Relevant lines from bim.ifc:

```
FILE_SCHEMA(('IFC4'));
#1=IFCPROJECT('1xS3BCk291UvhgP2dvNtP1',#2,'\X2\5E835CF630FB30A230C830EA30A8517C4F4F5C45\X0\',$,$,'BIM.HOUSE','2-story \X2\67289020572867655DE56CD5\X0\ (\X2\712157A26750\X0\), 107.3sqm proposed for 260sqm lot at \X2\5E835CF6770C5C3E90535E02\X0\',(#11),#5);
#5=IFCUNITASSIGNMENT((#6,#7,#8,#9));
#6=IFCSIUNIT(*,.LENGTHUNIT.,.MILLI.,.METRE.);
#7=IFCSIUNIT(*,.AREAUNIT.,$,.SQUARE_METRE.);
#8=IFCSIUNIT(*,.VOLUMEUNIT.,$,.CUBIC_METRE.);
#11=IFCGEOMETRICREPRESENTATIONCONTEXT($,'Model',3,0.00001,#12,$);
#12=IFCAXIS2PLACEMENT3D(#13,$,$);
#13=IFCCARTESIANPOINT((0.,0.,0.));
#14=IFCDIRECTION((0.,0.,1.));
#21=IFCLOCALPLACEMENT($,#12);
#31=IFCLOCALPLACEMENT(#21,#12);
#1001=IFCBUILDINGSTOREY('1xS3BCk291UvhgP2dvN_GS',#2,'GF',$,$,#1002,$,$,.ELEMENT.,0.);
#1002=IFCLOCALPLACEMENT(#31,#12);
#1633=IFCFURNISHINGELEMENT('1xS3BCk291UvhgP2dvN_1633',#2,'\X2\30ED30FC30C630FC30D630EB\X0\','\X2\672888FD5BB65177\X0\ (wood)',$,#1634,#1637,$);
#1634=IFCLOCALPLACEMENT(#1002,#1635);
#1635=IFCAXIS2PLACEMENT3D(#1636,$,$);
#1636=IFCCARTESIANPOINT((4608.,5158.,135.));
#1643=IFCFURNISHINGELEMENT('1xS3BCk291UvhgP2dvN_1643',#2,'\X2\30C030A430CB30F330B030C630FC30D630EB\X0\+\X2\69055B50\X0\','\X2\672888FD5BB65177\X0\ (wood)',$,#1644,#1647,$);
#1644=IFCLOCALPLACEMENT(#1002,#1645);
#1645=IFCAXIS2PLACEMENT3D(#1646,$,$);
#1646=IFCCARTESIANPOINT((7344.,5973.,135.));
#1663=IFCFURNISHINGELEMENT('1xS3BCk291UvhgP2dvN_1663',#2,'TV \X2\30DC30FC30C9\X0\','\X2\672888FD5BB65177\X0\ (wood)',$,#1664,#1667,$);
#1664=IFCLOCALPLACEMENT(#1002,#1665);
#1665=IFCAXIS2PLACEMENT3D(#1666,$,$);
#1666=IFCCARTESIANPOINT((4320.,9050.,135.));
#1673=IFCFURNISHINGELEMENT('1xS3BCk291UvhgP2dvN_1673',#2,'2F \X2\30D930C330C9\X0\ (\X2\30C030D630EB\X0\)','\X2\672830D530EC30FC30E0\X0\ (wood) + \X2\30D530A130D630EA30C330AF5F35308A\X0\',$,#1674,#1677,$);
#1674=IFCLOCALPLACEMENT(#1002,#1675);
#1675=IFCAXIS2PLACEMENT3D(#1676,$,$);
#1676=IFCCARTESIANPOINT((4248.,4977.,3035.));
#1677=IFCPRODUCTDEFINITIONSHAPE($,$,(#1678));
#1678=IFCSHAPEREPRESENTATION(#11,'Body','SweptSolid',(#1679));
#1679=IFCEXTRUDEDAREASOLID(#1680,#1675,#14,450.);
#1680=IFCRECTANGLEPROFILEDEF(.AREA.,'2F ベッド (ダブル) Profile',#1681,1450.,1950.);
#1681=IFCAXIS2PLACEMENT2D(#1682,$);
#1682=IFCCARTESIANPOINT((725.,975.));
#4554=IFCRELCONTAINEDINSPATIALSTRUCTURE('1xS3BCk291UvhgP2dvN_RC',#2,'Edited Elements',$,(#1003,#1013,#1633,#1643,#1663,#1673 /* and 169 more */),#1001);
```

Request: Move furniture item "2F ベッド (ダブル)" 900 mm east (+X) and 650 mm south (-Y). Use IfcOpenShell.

```python
import ifcopenshell
import ifcopenshell.api.geometry
import ifcopenshell.util.placement
import ifcopenshell.util.unit

model = ifcopenshell.open("bim.ifc")
unit_scale = ifcopenshell.util.unit.calculate_unit_scale(model)

item = model.by_guid("1xS3BCk291UvhgP2dvN_1673")
matrix = ifcopenshell.util.placement.get_local_placement(item.ObjectPlacement)
matrix[0, 3] += 0.9 / unit_scale
matrix[1, 3] -= 0.65 / unit_scale
ifcopenshell.api.geometry.edit_object_placement(model, product=item, matrix=matrix, is_si=False)

print(ifcopenshell.util.placement.get_local_placement(item.ObjectPlacement).round(3) + 0.0)

model.write("bim_edited.ifc")
```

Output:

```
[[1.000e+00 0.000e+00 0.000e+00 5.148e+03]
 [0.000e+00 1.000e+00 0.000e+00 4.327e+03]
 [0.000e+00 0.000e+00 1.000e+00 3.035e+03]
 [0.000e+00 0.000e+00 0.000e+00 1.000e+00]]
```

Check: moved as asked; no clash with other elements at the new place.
